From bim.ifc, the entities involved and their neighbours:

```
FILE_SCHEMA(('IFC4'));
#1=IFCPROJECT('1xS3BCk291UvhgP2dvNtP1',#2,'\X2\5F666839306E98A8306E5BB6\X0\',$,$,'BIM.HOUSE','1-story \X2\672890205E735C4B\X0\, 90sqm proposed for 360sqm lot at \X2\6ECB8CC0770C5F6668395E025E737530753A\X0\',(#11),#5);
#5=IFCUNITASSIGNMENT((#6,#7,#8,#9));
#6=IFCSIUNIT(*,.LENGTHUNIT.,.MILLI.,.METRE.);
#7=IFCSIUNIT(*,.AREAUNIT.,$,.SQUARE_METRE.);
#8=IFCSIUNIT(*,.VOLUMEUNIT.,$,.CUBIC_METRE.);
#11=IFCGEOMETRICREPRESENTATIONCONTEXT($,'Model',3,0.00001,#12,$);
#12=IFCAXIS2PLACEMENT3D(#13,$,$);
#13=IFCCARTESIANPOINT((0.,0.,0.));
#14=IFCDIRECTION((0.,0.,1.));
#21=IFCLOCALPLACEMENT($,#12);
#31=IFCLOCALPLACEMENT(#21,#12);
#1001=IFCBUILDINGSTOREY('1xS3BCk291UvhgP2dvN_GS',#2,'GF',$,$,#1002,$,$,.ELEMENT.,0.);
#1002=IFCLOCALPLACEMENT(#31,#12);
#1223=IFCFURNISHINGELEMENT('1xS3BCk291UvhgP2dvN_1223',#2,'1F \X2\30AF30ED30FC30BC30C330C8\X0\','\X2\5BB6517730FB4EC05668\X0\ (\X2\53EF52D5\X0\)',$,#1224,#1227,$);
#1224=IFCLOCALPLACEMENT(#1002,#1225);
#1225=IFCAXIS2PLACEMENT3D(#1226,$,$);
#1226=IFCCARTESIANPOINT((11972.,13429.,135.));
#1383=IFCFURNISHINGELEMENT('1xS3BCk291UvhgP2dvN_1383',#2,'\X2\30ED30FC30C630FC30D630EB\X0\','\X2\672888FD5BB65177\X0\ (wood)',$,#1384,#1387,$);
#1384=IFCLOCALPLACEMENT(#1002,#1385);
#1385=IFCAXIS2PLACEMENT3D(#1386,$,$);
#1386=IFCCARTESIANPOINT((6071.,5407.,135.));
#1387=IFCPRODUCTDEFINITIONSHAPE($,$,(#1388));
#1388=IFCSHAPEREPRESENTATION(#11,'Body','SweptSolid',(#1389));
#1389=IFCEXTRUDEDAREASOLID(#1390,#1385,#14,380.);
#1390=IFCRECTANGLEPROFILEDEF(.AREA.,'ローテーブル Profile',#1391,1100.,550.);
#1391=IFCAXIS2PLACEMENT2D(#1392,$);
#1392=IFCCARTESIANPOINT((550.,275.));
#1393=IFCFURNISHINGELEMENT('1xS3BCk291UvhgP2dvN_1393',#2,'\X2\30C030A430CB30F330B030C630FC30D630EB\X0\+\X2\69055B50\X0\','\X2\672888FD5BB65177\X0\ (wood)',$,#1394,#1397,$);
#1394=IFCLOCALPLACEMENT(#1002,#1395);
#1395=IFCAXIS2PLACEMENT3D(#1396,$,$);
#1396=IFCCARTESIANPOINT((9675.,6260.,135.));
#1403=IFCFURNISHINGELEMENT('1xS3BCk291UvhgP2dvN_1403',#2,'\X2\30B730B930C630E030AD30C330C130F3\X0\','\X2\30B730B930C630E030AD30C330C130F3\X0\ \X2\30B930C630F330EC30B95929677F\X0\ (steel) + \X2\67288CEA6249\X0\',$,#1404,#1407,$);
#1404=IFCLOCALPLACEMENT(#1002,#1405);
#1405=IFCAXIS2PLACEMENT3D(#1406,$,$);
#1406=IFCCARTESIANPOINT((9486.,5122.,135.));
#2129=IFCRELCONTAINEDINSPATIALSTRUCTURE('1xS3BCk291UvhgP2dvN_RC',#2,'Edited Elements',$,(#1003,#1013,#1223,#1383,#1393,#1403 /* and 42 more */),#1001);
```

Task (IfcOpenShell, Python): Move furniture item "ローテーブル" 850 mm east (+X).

```python
import ifcopenshell
import ifcopenshell.api.geometry
import ifcopenshell.util.placement
import ifcopenshell.util.unit

model = ifcopenshell.open("bim.ifc")
unit_scale = ifcopenshell.util.unit.calculate_unit_scale(model)

item = model.by_id(1383)
matrix = ifcopenshell.util.placement.get_local_placement(item.ObjectPlacement)
matrix[0, 3] += 0.85 / unit_scale
ifcopenshell.api.geometry.edit_object_placement(model, product=item, matrix=matrix, is_si=False)

print(ifcopenshell.util.placement.get_local_placement(item.ObjectPlacement).round(3) + 0.0)

model.write("bim_updated.ifc")
```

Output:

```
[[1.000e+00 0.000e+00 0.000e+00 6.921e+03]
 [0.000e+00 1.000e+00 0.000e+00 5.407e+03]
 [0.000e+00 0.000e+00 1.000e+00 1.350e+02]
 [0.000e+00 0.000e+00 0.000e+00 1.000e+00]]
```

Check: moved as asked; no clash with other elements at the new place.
